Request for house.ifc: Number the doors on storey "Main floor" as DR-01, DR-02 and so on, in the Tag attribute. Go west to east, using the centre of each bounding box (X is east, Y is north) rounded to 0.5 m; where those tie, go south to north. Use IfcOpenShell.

First a look at what the model holds.

```python
import ifcopenshell
import ifcopenshell.util.element
import ifcopenshell.util.placement

model = ifcopenshell.open("house.ifc")
print(model.schema)
storey = next(s for s in model.by_type("IfcBuildingStorey") if s.Name == "Main floor")
doors = [e for e in ifcopenshell.util.element.get_decomposition(storey) if e.is_a("IfcDoor")]
for e in sorted(doors, key=lambda e: e.id()):
    origin = ifcopenshell.util.placement.get_local_placement(e.ObjectPlacement)[:3, 3]
    print(e.id(), e.Tag, e.Name, origin.round(2) + 0.0, sep=" | ")
```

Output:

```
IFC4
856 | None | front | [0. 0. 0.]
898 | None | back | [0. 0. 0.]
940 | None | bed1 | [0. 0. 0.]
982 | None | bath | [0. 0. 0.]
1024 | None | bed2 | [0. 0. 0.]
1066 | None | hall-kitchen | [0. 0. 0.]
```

```python
import ifcopenshell
import ifcopenshell.geom
import ifcopenshell.util.element
import ifcopenshell.util.shape

model = ifcopenshell.open("house.ifc")
settings = ifcopenshell.geom.settings()
settings.set("use-world-coords", True)


def centre(element):
    shape = ifcopenshell.geom.create_shape(settings, element)
    return ifcopenshell.util.shape.get_bbox_centroid(shape.geometry)


storey = next(s for s in model.by_type("IfcBuildingStorey") if s.Name == "Main floor")
doors = [e for e in ifcopenshell.util.element.get_decomposition(storey) if e.is_a("IfcDoor")]

# Insertion points can sit at a corner or the storey origin, so sort by the geometry (in metres).
centres = {e: centre(e) for e in doors}
doors.sort(key=lambda e: (round(centres[e][0] / 0.5), centres[e][1]))

for i, e in enumerate(doors, start=1):
    number = f"DR-{i:02d}"
    e.Tag = number
    print(e.id(), number)

model.write("house_v2.ifc")
```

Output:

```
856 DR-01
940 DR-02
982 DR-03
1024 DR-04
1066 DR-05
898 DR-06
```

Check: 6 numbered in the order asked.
